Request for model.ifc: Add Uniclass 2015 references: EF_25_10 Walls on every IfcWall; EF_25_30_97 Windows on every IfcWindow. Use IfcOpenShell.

First a look at what the model holds.

```python
import ifcopenshell

model = ifcopenshell.open("model.ifc")
print(model.schema)
print("classifications:", [c.Name for c in model.by_type("IfcClassification")])
for ifc_class in ("IfcDoor", "IfcRoof", "IfcStair", "IfcWall", "IfcWindow"):
    print(ifc_class, len(model.by_type(ifc_class)))
```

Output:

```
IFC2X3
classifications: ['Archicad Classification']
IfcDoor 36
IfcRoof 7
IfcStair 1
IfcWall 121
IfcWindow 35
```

```python
import ifcopenshell
import ifcopenshell.api.classification

model = ifcopenshell.open("model.ifc")

# IFC2X3 requires Source and Edition and has no link from the project to the system.
system = model.create_entity("IfcClassification", Source="NBS", Edition="2015", Name="Uniclass 2015")

codes = {
    "IfcWall": ("EF_25_10", "Walls"),
    "IfcWindow": ("EF_25_30_97", "Windows"),
}
for ifc_class, (code, name) in codes.items():
    products = model.by_type(ifc_class)
    ifcopenshell.api.classification.add_reference(
        model, products=products, classification=system, identification=code, name=name
    )
    print(code, len(products))

model.write("model-out.ifc")
```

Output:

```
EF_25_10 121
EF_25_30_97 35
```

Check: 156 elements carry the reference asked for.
